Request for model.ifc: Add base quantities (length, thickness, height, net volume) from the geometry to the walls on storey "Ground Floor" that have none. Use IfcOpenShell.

First a look at what the model holds.

```python
import ifcopenshell
import ifcopenshell.util.element
import ifcopenshell.util.unit

model = ifcopenshell.open("model.ifc")
print(model.schema)
for unit_type in ("LENGTHUNIT", "AREAUNIT", "VOLUMEUNIT"):
    print(unit_type, ifcopenshell.util.unit.calculate_unit_scale(model, unit_type))
storey = next(s for s in model.by_type("IfcBuildingStorey") if s.Name == "Ground Floor")
walls = [e for e in ifcopenshell.util.element.get_decomposition(storey) if e.is_a("IfcWall")]
for e in sorted(walls, key=lambda e: e.id()):
    print(e.id(), e.is_a(), e.Name, list(ifcopenshell.util.element.get_psets(e, qtos_only=True)), sep=" | ")
```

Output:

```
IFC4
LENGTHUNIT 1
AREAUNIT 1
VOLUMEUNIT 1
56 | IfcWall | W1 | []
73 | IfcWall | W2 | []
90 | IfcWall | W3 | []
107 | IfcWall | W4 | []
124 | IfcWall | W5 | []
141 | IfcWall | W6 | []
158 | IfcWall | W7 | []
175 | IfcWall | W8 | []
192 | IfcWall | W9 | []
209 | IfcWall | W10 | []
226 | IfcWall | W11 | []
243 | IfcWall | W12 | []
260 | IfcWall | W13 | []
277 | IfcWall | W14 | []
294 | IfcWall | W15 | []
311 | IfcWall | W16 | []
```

```python
import ifcopenshell
import ifcopenshell.api.pset
import ifcopenshell.geom
import ifcopenshell.util.element
import ifcopenshell.util.shape
import ifcopenshell.util.unit

model = ifcopenshell.open("model.ifc")
unit_scale = ifcopenshell.util.unit.calculate_unit_scale(model)
volume_scale = ifcopenshell.util.unit.calculate_unit_scale(model, "VOLUMEUNIT")
settings = ifcopenshell.geom.settings()

storey = next(s for s in model.by_type("IfcBuildingStorey") if s.Name == "Ground Floor")
walls = [e for e in ifcopenshell.util.element.get_decomposition(storey) if e.is_a("IfcWall")]

for e in sorted(walls, key=lambda e: e.id()):
    if ifcopenshell.util.element.get_psets(e, qtos_only=True, should_inherit=False):
        continue
    # Geometry comes back in metres, in the element's own axes.
    shape = ifcopenshell.geom.create_shape(settings, e)
    values = {
        "Length": ifcopenshell.util.shape.get_x(shape.geometry) / unit_scale,
        "Width": ifcopenshell.util.shape.get_y(shape.geometry) / unit_scale,
        "Height": ifcopenshell.util.shape.get_z(shape.geometry) / unit_scale,
        "NetVolume": ifcopenshell.util.shape.get_volume(shape.geometry) / volume_scale,
    }
    qto = ifcopenshell.api.pset.add_qto(model, product=e, name="Qto_WallBaseQuantities")
    ifcopenshell.api.pset.edit_qto(model, qto=qto, properties=values)
    print(e.id(), {k: round(v, 3) for k, v in values.items()})

model.write("model_v2.ifc")
```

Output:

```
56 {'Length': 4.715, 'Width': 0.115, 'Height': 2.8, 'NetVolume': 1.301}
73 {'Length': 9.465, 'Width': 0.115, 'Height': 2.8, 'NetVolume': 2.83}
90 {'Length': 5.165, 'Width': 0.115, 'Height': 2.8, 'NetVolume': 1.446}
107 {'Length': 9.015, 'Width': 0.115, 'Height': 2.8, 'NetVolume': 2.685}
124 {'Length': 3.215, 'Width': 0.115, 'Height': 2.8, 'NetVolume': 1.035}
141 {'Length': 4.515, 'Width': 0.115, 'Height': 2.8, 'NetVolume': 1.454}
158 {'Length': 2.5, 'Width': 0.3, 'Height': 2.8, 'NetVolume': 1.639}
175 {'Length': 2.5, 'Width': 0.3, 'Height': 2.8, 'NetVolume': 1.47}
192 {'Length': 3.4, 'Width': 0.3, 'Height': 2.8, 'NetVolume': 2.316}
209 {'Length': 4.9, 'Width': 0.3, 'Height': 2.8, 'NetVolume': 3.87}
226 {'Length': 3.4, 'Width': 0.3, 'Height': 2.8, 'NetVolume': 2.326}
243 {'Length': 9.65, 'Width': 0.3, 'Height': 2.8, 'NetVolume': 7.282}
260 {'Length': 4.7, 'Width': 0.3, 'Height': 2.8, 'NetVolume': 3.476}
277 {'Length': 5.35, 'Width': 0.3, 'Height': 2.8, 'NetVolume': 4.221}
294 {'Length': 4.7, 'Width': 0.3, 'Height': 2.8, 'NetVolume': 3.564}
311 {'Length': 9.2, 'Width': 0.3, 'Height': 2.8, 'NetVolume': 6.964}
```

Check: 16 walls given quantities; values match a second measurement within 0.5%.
